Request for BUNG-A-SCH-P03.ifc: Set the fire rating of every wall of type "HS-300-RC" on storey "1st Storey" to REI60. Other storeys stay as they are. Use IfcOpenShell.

First a look at what the model holds.

```python
import ifcopenshell
import ifcopenshell.util.element

model = ifcopenshell.open("BUNG-A-SCH-P03.ifc")
print(model.schema)
storey = next(s for s in model.by_type("IfcBuildingStorey") if s.Name == "1st Storey")
walls = [e for e in ifcopenshell.util.element.get_decomposition(storey) if e.is_a("IfcWall")]
seen = {}
for e in walls:
    element_type = ifcopenshell.util.element.get_type(e)
    key = (element_type.Name if element_type != e and element_type else None, ifcopenshell.util.element.get_pset(e, "Pset_WallCommon", "FireRating"))
    seen[key] = seen.get(key, 0) + 1
for (name, value), count in sorted(seen.items(), key=str):
    print(count, "x", name, "|", value)
```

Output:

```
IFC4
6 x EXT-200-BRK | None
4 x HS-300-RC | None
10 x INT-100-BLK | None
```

```python
import ifcopenshell
import ifcopenshell.api.pset
import ifcopenshell.util.element

model = ifcopenshell.open("BUNG-A-SCH-P03.ifc")

storey = next(s for s in model.by_type("IfcBuildingStorey") if s.Name == "1st Storey")
walls = [e for e in ifcopenshell.util.element.get_decomposition(storey) if e.is_a("IfcWall")]

count = 0
for e in walls:
    element_type = ifcopenshell.util.element.get_type(e)
    if element_type in (None, e) or element_type.Name != "HS-300-RC":
        continue
    # add_pset returns the element's existing set when there is one.
    pset = ifcopenshell.api.pset.add_pset(model, product=e, name="Pset_WallCommon")
    ifcopenshell.api.pset.edit_pset(model, pset=pset, properties={"FireRating": "REI60"})
    count += 1

print(count, "walls updated")

model.write("BUNG-A-SCH-P03_edited.ifc")
```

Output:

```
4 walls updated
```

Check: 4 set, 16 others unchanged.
